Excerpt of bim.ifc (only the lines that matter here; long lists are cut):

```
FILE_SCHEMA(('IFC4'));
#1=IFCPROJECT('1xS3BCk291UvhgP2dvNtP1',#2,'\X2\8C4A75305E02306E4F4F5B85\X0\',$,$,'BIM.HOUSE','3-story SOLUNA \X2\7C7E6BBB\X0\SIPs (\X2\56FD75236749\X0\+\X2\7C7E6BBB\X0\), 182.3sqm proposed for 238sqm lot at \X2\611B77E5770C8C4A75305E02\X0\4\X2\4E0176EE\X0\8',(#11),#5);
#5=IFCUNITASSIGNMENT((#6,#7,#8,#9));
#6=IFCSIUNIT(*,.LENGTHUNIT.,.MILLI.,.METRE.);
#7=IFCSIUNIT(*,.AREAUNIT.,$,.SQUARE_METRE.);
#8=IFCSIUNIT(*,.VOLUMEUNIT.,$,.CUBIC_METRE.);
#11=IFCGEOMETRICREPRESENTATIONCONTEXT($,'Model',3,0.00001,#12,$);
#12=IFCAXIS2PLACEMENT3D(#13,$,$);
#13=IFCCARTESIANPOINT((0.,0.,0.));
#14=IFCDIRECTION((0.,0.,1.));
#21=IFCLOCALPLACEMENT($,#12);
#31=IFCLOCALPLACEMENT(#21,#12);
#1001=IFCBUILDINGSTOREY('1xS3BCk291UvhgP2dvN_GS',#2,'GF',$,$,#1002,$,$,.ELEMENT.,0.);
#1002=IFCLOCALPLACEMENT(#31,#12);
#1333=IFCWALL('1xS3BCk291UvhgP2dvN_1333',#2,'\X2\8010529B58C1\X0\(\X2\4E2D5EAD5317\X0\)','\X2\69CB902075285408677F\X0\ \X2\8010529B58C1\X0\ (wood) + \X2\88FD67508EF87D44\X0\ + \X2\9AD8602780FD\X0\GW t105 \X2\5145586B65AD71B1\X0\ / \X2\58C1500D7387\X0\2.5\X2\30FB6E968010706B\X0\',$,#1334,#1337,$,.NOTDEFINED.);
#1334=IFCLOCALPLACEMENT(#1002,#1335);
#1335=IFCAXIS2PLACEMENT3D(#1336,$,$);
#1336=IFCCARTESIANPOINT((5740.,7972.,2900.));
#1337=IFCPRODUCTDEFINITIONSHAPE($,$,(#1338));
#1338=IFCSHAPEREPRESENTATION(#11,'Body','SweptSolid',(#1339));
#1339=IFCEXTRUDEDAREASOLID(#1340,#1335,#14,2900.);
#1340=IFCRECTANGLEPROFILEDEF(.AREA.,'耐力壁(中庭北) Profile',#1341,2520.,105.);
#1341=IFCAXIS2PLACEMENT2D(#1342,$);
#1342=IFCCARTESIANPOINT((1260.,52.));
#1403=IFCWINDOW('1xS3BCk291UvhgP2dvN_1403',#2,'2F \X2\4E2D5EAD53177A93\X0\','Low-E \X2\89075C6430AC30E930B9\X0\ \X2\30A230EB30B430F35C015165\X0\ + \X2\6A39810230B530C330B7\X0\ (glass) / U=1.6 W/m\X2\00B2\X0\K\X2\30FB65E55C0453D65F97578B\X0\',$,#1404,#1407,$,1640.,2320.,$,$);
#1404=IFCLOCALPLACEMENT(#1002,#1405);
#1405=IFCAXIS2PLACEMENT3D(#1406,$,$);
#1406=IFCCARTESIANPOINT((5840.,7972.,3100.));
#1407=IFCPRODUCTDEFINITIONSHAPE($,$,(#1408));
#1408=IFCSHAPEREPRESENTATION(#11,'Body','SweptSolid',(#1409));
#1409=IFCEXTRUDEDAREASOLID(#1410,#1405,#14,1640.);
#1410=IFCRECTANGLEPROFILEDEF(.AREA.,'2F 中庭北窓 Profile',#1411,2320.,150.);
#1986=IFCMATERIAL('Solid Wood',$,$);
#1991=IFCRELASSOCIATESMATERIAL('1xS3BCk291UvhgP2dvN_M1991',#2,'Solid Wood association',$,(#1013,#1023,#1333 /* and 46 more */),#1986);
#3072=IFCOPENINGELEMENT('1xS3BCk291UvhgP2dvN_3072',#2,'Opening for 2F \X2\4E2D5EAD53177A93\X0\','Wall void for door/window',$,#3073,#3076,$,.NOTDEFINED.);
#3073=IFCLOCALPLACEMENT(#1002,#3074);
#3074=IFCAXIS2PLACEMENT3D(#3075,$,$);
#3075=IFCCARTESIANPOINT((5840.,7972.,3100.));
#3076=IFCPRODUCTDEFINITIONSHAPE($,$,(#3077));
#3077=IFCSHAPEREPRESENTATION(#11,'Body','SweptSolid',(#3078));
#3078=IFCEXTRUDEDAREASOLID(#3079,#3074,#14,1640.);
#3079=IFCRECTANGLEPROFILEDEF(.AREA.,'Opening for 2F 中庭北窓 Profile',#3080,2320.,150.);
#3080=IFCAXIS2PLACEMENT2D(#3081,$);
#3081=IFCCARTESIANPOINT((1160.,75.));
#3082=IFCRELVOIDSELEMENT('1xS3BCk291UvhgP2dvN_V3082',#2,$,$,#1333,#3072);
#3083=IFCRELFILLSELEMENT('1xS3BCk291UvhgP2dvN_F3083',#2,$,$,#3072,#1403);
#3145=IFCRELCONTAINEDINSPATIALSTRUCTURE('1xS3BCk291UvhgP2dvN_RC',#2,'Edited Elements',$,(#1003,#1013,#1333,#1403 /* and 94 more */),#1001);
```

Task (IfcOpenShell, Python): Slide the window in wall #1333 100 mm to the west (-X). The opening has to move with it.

```python
import ifcopenshell
import ifcopenshell.api.geometry
import ifcopenshell.util.placement

model = ifcopenshell.open("bim.ifc")

window = model.by_id(1403)
opening = window.FillsVoids[0].RelatingOpeningElement
wall = opening.VoidsElements[0].RelatingBuildingElement

wall_matrix = ifcopenshell.util.placement.get_local_placement(wall.ObjectPlacement)
shift = wall_matrix[:3, 0] * -100.0
before = ifcopenshell.util.placement.get_local_placement(window.ObjectPlacement)[:3, 3].copy()

# The window is not placed relative to its opening, so move both.
for product in (opening, window):
    matrix = ifcopenshell.util.placement.get_local_placement(product.ObjectPlacement)
    matrix[:3, 3] += shift
    ifcopenshell.api.geometry.edit_object_placement(model, product=product, matrix=matrix, is_si=False)

after = ifcopenshell.util.placement.get_local_placement(window.ObjectPlacement)[:3, 3]
print("window moved by", (after - before).round(3) + 0.0)

model.write("bim_updated.ifc")
```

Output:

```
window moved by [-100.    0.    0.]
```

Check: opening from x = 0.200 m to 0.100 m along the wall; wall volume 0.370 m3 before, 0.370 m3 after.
